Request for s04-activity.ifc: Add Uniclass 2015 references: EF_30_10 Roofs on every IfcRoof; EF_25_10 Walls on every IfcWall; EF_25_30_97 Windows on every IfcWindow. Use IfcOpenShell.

First a look at what the model holds.

```python
import ifcopenshell

model = ifcopenshell.open("s04-activity.ifc")
print(model.schema)
print("classifications:", [c.Name for c in model.by_type("IfcClassification")])
for ifc_class in ("IfcDoor", "IfcRoof", "IfcStair", "IfcWall", "IfcWindow"):
    print(ifc_class, len(model.by_type(ifc_class)))
```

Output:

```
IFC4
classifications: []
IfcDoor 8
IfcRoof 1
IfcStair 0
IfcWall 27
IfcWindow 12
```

```python
import ifcopenshell
import ifcopenshell.api.classification

model = ifcopenshell.open("s04-activity.ifc")

system = ifcopenshell.api.classification.add_classification(model, classification="Uniclass 2015")

codes = {
    "IfcRoof": ("EF_30_10", "Roofs"),
    "IfcWall": ("EF_25_10", "Walls"),
    "IfcWindow": ("EF_25_30_97", "Windows"),
}
for ifc_class, (code, name) in codes.items():
    products = model.by_type(ifc_class)
    ifcopenshell.api.classification.add_reference(
        model, products=products, classification=system, identification=code, name=name
    )
    print(code, len(products))

model.write("s04-activity-out.ifc")
```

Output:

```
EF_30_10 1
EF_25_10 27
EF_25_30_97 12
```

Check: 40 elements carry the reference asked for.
